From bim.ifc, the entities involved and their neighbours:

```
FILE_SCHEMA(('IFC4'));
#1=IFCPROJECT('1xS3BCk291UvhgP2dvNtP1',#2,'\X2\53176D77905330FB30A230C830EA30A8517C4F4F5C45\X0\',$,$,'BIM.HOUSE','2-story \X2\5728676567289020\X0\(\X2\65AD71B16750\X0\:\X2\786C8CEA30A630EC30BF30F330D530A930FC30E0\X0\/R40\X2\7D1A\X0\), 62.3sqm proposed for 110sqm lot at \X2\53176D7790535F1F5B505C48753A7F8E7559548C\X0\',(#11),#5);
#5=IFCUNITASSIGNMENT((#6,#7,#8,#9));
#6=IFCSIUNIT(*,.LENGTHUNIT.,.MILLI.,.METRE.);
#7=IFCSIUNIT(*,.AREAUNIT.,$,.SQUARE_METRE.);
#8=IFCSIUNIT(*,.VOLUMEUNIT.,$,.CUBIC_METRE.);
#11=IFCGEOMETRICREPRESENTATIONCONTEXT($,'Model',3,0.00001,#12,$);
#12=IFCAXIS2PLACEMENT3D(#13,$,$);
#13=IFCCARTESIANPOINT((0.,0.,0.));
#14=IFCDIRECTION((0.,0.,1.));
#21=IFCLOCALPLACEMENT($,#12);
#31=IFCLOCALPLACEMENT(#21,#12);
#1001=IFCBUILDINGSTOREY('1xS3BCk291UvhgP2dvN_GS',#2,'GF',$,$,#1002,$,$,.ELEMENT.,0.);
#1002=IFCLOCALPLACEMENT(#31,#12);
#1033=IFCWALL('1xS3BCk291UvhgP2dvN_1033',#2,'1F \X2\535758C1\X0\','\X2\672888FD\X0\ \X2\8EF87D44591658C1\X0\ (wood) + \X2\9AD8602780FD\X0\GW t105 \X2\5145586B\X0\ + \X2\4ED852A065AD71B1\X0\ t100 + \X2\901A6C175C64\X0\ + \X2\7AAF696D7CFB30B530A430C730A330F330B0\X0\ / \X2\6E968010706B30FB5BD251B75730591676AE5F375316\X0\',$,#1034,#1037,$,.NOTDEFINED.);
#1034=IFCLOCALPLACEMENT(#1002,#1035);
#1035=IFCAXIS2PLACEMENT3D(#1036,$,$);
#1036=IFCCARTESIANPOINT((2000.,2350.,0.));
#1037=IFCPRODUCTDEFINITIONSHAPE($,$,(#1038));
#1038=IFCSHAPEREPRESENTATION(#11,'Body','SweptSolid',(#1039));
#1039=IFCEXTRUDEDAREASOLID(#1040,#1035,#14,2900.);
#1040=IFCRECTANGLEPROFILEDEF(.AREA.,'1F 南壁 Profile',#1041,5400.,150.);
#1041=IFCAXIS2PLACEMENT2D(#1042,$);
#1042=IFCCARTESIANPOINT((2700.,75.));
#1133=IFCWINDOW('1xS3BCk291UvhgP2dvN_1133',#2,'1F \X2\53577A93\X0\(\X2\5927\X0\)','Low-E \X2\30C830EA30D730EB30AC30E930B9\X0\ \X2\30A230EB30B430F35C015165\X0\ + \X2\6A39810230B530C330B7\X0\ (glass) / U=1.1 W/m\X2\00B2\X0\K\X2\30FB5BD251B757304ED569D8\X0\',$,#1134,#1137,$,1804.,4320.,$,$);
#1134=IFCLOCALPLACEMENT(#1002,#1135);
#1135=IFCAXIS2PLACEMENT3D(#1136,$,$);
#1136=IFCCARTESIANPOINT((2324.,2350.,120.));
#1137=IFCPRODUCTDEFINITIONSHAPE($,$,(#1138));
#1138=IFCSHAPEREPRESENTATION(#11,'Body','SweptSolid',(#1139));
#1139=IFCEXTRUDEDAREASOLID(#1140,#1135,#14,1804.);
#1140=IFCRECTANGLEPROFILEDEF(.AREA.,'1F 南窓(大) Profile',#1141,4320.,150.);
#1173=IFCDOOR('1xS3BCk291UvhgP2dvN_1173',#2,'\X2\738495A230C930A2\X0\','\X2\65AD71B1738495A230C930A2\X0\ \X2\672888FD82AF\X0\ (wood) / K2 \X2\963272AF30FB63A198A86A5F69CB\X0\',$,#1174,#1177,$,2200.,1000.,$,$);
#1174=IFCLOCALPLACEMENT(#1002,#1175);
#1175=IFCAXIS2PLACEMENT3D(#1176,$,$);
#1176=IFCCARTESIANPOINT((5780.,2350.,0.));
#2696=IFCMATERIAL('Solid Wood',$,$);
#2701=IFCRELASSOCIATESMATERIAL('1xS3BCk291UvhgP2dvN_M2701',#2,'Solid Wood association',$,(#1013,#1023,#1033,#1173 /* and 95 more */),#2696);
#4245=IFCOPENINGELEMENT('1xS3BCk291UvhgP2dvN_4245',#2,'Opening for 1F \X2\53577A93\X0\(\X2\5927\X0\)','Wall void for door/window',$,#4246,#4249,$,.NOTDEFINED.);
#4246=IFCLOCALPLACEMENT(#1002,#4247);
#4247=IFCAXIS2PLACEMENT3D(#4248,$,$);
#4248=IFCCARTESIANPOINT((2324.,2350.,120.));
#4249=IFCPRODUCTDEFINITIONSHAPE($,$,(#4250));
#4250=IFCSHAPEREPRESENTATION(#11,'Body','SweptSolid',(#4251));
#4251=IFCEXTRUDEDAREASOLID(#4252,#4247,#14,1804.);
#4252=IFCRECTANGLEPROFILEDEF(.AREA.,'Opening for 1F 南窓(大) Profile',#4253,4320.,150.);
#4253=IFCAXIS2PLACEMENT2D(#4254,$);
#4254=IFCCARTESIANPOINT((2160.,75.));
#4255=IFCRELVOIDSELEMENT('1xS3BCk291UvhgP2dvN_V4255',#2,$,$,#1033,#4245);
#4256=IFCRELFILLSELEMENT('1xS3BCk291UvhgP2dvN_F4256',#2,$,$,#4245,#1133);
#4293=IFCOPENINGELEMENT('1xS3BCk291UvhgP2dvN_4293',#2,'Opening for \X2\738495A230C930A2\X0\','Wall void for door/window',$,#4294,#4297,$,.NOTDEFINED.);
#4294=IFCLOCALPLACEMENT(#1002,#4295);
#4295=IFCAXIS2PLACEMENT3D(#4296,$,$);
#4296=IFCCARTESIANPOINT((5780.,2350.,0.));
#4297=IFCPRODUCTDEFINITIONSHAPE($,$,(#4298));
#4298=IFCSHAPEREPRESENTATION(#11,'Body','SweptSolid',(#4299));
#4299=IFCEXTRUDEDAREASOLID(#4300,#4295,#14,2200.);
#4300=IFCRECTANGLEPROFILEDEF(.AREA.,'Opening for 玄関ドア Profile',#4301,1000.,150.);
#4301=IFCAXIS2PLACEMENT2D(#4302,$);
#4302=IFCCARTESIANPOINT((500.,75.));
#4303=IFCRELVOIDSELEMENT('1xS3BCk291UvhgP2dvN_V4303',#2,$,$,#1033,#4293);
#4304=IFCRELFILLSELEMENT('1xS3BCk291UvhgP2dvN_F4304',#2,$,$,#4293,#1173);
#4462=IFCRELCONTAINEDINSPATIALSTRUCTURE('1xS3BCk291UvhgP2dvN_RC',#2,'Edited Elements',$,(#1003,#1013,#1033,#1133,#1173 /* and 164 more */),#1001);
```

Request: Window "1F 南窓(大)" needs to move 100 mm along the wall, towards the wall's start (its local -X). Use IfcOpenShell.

```python
import ifcopenshell
import ifcopenshell.api.geometry
import ifcopenshell.util.placement

model = ifcopenshell.open("bim.ifc")

window = model.by_id(1133)
opening = window.FillsVoids[0].RelatingOpeningElement
wall = opening.VoidsElements[0].RelatingBuildingElement

wall_matrix = ifcopenshell.util.placement.get_local_placement(wall.ObjectPlacement)
shift = wall_matrix[:3, 0] * -100.0
before = ifcopenshell.util.placement.get_local_placement(window.ObjectPlacement)[:3, 3].copy()

# The window is not placed relative to its opening, so move both.
for product in (opening, window):
    matrix = ifcopenshell.util.placement.get_local_placement(product.ObjectPlacement)
    matrix[:3, 3] += shift
    ifcopenshell.api.geometry.edit_object_placement(model, product=product, matrix=matrix, is_si=False)

after = ifcopenshell.util.placement.get_local_placement(window.ObjectPlacement)[:3, 3]
print("window moved by", (after - before).round(3) + 0.0)

model.write("bim_edited.ifc")
```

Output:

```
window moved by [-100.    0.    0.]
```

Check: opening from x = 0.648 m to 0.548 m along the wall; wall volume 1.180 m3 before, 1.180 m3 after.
